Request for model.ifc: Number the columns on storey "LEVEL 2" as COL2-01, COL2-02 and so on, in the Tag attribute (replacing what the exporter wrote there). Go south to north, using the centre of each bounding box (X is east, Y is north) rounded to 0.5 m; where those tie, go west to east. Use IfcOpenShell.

First a look at what the model holds.

```python
import ifcopenshell
import ifcopenshell.util.element
import ifcopenshell.util.placement

model = ifcopenshell.open("model.ifc")
print(model.schema)
storey = next(s for s in model.by_type("IfcBuildingStorey") if s.Name == "LEVEL 2")
columns = [e for e in ifcopenshell.util.element.get_decomposition(storey) if e.is_a("IfcColumn")]
for e in sorted(columns, key=lambda e: e.id()):
    origin = ifcopenshell.util.placement.get_local_placement(e.ObjectPlacement)[:3, 3]
    print(e.id(), e.Tag, e.Name, origin.round(2) + 0.0, sep=" | ")
```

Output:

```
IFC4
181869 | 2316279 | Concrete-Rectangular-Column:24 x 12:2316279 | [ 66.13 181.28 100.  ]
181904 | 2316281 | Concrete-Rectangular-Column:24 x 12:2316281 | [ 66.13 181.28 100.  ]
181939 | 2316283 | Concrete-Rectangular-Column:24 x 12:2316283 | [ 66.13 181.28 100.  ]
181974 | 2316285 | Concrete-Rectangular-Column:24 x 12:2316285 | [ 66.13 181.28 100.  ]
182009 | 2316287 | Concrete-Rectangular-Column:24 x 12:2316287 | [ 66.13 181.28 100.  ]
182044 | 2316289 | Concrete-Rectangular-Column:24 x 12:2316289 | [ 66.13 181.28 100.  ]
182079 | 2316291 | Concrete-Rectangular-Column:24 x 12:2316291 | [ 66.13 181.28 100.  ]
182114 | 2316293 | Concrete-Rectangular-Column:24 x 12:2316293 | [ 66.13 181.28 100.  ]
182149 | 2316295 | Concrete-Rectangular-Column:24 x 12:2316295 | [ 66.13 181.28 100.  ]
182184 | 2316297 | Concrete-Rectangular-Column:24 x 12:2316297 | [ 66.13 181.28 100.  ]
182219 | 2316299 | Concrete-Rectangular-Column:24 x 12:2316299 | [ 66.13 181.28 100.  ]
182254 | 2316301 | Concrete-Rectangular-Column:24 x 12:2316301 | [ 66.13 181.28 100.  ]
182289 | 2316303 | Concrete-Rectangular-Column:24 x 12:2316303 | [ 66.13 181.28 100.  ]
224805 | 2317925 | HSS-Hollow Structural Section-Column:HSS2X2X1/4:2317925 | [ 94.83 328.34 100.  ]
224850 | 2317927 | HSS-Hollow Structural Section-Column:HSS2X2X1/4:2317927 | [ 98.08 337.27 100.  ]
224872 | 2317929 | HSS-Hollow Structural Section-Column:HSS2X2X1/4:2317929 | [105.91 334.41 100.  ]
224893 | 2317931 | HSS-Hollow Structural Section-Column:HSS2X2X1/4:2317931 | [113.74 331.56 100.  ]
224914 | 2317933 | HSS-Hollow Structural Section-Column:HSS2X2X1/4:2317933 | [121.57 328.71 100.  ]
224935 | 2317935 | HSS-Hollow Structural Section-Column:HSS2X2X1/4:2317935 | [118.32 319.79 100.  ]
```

```python
import ifcopenshell
import ifcopenshell.geom
import ifcopenshell.util.element
import ifcopenshell.util.shape

model = ifcopenshell.open("model.ifc")
settings = ifcopenshell.geom.settings()
settings.set("use-world-coords", True)


def centre(element):
    shape = ifcopenshell.geom.create_shape(settings, element)
    return ifcopenshell.util.shape.get_bbox_centroid(shape.geometry)


storey = next(s for s in model.by_type("IfcBuildingStorey") if s.Name == "LEVEL 2")
columns = [e for e in ifcopenshell.util.element.get_decomposition(storey) if e.is_a("IfcColumn")]

# Insertion points can sit at a corner or the storey origin, so sort by the geometry (in metres).
centres = {e: centre(e) for e in columns}
columns.sort(key=lambda e: (round(centres[e][1] / 0.5), centres[e][0]))

for i, e in enumerate(columns, start=1):
    number = f"COL2-{i:02d}"
    e.Tag = number
    print(e.id(), number)

model.write("model_v2.ifc")
```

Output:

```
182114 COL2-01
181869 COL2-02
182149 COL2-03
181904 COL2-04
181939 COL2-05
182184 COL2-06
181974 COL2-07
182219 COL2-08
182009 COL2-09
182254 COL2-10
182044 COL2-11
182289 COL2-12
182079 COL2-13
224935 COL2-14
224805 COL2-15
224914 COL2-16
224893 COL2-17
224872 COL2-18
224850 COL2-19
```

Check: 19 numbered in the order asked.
